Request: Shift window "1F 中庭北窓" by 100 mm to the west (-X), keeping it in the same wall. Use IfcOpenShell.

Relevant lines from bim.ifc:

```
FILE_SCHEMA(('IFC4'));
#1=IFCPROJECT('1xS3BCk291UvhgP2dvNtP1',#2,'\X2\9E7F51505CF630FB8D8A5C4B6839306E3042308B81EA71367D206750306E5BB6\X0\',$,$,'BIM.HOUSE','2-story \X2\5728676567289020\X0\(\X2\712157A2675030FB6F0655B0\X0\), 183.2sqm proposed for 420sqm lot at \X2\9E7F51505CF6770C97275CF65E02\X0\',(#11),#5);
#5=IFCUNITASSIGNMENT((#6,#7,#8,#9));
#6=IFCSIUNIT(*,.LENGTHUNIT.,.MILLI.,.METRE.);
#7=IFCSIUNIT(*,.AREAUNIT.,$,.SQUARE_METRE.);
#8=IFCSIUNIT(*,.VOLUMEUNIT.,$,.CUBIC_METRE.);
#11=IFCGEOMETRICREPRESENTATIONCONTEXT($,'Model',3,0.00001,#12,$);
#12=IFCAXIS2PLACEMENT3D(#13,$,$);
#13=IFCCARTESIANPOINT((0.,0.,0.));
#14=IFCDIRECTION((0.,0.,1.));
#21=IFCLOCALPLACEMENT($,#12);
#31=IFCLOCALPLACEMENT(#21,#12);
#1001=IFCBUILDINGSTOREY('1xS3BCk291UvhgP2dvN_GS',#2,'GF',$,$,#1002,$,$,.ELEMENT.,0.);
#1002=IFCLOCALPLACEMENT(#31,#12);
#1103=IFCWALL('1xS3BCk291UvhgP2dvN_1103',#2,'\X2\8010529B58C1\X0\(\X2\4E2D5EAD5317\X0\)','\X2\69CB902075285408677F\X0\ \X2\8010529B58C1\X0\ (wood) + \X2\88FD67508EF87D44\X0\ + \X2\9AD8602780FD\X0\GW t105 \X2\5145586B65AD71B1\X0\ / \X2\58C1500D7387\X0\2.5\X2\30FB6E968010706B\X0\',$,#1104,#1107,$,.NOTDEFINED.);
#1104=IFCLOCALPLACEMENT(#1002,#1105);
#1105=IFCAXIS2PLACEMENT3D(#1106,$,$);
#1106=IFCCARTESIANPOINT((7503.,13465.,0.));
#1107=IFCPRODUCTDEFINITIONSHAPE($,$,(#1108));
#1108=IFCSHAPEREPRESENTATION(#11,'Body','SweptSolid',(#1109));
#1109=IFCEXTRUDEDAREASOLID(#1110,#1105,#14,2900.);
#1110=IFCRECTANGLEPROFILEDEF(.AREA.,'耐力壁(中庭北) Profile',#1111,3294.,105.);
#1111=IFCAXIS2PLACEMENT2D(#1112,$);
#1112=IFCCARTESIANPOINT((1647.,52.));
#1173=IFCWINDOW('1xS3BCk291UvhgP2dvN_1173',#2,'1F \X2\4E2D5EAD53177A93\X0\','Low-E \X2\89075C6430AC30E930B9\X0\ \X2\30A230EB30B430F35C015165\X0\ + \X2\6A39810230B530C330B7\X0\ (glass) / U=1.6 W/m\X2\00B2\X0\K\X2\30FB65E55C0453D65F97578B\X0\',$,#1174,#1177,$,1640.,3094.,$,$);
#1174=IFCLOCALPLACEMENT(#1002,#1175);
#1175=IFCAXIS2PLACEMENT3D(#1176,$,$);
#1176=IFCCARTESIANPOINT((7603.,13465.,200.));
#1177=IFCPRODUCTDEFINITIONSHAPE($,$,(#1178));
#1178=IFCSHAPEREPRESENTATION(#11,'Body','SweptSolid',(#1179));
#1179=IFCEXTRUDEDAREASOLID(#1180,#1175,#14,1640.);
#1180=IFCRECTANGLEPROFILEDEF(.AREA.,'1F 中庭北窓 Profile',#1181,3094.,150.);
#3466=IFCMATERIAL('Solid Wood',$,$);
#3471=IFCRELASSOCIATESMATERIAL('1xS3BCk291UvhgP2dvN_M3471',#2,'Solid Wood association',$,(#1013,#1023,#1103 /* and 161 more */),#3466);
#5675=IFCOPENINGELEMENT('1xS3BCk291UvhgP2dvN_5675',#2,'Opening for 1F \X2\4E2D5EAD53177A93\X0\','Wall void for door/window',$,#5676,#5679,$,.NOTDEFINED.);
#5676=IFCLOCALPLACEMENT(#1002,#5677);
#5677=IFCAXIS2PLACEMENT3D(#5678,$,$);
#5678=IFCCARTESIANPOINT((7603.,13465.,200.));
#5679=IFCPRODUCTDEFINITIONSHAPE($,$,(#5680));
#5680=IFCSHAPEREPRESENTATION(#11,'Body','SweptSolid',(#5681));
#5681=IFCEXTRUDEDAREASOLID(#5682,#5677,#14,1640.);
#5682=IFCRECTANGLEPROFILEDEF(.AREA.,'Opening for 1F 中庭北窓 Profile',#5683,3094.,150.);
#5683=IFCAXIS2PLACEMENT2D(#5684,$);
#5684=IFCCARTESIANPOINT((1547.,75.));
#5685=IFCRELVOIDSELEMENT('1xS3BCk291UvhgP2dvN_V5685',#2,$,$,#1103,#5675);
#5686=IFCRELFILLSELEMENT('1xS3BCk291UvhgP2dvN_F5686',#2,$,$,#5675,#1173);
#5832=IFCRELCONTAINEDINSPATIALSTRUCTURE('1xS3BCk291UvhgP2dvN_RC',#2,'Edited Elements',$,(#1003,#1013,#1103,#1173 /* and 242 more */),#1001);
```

```python
import ifcopenshell
import ifcopenshell.api.geometry
import ifcopenshell.util.placement
import ifcopenshell.util.unit

model = ifcopenshell.open("bim.ifc")
unit_scale = ifcopenshell.util.unit.calculate_unit_scale(model)

window = model.by_id(1173)
opening = window.FillsVoids[0].RelatingOpeningElement
wall = opening.VoidsElements[0].RelatingBuildingElement

wall_matrix = ifcopenshell.util.placement.get_local_placement(wall.ObjectPlacement)
shift = wall_matrix[:3, 0] * -0.1 / unit_scale
before = ifcopenshell.util.placement.get_local_placement(window.ObjectPlacement)[:3, 3].copy()

# The window is not placed relative to its opening, so move both.
for product in (opening, window):
    matrix = ifcopenshell.util.placement.get_local_placement(product.ObjectPlacement)
    matrix[:3, 3] += shift
    ifcopenshell.api.geometry.edit_object_placement(model, product=product, matrix=matrix, is_si=False)

after = ifcopenshell.util.placement.get_local_placement(window.ObjectPlacement)[:3, 3]
print("window moved by", (after - before).round(3) + 0.0)

model.write("bim_edited.ifc")
```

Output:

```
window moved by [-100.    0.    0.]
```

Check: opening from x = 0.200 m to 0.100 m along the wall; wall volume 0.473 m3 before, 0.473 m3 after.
